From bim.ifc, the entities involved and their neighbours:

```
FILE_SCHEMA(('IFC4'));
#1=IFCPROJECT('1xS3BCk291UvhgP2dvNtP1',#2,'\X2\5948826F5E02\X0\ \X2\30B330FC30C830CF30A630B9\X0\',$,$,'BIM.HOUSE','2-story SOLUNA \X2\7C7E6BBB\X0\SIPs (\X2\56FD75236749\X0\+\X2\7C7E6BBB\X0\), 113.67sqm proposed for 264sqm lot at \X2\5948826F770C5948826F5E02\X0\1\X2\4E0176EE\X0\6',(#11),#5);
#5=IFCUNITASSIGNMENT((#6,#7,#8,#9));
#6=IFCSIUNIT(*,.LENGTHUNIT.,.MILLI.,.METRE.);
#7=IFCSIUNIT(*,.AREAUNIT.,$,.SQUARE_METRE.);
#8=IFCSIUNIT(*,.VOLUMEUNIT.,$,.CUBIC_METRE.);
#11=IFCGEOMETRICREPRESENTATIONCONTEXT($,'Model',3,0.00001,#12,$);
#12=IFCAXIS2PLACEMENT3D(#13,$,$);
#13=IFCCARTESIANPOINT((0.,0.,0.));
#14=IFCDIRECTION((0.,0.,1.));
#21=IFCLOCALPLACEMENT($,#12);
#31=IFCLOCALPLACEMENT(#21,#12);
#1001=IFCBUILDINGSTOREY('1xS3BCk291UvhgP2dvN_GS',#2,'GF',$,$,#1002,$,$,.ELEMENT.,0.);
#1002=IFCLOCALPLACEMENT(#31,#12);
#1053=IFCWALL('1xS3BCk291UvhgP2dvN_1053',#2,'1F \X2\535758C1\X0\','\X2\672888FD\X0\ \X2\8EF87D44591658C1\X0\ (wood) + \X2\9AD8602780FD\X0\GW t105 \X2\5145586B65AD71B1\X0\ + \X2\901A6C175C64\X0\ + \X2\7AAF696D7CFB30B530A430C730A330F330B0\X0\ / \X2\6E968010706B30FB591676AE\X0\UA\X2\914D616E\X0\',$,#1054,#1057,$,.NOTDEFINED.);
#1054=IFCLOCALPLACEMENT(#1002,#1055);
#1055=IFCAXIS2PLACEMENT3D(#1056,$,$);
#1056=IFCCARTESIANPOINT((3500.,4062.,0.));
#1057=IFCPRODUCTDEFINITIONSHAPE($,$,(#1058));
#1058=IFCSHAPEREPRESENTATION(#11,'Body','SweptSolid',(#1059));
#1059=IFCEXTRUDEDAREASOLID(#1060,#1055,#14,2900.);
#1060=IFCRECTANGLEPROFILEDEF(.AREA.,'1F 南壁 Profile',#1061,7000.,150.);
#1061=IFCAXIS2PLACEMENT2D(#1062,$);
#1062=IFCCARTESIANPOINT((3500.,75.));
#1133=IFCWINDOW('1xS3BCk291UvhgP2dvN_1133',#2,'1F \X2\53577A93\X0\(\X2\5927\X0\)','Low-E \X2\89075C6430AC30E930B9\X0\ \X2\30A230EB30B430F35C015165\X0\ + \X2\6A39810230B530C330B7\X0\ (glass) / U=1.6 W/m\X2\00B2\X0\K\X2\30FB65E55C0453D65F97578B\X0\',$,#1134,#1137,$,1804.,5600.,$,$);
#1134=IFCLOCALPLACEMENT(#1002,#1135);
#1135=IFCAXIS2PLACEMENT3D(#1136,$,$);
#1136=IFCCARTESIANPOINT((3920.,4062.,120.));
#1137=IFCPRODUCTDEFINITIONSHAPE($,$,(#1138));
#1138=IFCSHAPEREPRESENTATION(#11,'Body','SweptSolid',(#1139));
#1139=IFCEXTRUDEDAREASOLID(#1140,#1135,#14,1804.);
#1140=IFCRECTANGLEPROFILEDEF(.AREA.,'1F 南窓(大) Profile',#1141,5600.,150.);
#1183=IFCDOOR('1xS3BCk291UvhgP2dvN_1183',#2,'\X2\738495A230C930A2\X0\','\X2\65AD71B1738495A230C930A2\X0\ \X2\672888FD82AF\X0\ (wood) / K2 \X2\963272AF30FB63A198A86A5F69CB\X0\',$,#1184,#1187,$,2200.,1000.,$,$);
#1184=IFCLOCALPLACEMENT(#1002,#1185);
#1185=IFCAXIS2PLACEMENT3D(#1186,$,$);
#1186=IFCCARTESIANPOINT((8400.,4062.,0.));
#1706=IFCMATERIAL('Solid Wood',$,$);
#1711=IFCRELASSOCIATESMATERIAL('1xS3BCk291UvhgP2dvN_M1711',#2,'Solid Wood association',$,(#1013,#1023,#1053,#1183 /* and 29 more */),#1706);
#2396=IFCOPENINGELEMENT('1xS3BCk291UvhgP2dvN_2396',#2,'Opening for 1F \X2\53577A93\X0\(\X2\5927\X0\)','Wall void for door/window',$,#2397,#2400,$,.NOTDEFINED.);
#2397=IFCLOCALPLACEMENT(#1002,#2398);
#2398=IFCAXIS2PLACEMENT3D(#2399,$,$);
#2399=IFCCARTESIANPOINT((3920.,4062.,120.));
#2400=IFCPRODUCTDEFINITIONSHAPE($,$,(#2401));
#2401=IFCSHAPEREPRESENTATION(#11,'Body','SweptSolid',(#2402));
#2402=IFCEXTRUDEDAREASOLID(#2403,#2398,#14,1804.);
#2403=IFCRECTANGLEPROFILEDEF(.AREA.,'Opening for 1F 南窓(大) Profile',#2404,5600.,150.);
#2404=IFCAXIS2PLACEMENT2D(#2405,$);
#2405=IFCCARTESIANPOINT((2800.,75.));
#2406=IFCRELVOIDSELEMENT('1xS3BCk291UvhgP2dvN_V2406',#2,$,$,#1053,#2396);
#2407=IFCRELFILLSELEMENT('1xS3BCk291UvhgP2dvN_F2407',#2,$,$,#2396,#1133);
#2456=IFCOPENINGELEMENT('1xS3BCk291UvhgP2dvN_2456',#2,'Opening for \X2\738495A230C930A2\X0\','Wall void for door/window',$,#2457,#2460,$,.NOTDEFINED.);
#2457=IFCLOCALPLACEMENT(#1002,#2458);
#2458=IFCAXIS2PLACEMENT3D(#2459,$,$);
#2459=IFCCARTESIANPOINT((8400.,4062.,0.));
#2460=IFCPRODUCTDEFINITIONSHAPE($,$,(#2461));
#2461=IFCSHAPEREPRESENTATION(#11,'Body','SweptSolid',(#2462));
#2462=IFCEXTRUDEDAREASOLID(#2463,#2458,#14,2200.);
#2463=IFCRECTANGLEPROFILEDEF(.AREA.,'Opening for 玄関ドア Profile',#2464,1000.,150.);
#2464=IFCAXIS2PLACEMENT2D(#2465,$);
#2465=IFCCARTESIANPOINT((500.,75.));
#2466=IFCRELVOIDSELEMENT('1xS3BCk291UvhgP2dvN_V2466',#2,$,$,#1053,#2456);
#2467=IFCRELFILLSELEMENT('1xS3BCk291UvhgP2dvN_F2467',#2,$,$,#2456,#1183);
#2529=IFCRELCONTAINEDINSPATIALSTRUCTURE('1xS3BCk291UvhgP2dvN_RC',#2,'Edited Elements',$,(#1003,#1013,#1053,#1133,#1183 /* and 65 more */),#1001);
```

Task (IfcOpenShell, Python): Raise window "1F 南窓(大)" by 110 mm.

```python
import numpy as np
import ifcopenshell
import ifcopenshell.api.geometry
import ifcopenshell.util.placement
import ifcopenshell.util.unit

model = ifcopenshell.open("bim.ifc")
unit_scale = ifcopenshell.util.unit.calculate_unit_scale(model)

window = model.by_id(1133)
opening = window.FillsVoids[0].RelatingOpeningElement
dz = 0.11 / unit_scale

shift = np.array([0.0, 0.0, dz])
# The window is not placed relative to its opening, so move both.
for product in (opening, window):
    matrix = ifcopenshell.util.placement.get_local_placement(product.ObjectPlacement)
    matrix[:3, 3] += shift
    ifcopenshell.api.geometry.edit_object_placement(model, product=product, matrix=matrix, is_si=False)

print(f"moved by {dz * unit_scale:+.3f} m")

model.write("bim_rev.ifc")
```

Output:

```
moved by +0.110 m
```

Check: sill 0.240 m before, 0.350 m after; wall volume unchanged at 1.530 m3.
